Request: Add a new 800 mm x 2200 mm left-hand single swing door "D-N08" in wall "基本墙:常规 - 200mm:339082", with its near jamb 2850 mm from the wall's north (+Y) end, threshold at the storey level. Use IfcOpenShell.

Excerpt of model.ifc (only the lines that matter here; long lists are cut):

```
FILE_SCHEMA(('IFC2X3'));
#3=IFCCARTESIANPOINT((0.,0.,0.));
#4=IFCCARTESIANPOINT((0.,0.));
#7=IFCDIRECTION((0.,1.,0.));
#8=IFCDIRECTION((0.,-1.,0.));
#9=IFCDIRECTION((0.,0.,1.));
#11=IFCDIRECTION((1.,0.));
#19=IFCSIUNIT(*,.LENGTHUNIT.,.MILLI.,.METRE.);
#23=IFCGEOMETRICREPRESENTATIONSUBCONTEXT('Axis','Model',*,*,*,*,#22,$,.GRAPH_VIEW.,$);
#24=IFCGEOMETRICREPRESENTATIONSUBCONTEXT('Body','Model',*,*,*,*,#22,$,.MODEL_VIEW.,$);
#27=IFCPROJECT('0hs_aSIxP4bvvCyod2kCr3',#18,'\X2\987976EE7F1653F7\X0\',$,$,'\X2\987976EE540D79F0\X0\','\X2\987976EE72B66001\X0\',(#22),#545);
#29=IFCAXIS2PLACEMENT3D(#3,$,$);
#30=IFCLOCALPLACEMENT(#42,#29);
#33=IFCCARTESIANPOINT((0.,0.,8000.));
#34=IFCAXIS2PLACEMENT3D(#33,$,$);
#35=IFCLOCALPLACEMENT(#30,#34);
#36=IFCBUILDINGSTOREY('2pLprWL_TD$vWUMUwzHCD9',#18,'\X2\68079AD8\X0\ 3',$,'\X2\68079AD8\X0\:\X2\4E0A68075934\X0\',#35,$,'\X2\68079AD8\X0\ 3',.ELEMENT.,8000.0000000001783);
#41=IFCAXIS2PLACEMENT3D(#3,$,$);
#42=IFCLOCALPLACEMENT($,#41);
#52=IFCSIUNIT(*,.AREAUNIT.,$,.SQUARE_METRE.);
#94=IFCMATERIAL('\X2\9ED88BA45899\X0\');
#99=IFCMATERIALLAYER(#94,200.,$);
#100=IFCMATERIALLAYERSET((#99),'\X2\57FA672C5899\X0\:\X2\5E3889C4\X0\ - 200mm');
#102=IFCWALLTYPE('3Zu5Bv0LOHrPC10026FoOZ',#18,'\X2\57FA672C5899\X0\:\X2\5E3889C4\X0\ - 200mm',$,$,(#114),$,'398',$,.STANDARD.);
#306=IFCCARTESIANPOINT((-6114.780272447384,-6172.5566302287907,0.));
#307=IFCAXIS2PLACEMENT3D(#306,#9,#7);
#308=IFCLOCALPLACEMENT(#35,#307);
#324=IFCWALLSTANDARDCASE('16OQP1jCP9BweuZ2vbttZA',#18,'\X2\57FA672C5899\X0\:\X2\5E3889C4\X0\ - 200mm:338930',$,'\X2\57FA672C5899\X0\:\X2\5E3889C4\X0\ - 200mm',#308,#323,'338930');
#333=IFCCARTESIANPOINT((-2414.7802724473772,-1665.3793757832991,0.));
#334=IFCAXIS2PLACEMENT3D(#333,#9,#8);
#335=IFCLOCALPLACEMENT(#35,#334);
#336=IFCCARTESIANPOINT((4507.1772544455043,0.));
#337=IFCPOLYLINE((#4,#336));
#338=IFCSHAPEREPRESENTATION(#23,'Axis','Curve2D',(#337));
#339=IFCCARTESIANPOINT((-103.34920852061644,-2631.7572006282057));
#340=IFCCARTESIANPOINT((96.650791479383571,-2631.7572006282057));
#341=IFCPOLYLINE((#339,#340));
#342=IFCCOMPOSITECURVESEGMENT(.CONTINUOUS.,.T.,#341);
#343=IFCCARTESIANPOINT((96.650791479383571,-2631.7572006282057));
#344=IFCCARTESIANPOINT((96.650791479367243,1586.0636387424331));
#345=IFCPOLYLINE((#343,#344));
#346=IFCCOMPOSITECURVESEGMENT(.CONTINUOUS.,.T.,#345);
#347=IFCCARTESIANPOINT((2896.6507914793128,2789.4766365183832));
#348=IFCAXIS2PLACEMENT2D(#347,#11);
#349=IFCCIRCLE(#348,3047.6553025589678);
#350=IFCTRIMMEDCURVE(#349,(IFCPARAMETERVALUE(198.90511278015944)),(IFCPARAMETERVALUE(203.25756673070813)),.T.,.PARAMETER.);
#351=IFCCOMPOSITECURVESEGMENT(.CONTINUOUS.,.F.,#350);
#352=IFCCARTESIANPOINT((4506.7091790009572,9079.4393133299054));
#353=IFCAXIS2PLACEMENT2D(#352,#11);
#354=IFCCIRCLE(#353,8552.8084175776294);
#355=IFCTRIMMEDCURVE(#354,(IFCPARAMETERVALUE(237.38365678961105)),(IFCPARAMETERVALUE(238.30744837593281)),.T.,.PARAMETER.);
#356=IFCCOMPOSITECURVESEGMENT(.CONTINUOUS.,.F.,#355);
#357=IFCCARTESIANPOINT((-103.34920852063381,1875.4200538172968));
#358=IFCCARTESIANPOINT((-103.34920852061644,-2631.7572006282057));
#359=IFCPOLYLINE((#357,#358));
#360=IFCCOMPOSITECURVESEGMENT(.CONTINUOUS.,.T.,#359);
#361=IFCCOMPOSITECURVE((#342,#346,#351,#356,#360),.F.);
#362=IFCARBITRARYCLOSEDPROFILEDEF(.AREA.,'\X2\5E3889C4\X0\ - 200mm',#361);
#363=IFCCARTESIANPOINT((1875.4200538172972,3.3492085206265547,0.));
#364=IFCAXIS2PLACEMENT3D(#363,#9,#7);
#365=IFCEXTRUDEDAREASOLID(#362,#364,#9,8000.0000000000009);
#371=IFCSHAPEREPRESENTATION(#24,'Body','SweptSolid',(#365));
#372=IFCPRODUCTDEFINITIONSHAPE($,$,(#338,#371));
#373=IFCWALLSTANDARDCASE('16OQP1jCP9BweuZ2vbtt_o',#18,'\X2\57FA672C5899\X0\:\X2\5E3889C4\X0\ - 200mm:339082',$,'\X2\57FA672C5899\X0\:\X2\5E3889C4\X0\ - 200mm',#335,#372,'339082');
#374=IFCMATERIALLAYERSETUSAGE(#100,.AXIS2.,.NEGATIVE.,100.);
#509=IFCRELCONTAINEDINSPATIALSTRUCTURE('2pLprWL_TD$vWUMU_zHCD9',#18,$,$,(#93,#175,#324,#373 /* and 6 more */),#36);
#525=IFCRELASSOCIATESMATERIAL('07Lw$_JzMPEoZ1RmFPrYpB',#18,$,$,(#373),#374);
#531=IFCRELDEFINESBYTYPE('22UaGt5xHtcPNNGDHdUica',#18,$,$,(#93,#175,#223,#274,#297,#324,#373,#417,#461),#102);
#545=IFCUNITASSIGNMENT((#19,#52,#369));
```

```python
import numpy as np
import ifcopenshell
import ifcopenshell.api.feature
import ifcopenshell.api.geometry
import ifcopenshell.api.root
import ifcopenshell.api.spatial
import ifcopenshell.api.type
import ifcopenshell.geom
import ifcopenshell.util.element
import ifcopenshell.util.placement
import ifcopenshell.util.representation
import ifcopenshell.util.shape
import ifcopenshell.util.unit

model = ifcopenshell.open("model.ifc")
unit_scale = ifcopenshell.util.unit.calculate_unit_scale(model)
settings = ifcopenshell.geom.settings()


def volume(element):
    """Net volume in cubic metres, openings subtracted."""
    shape = ifcopenshell.geom.create_shape(settings, element)
    return ifcopenshell.util.shape.get_volume(shape.geometry)


wall = model.by_guid("16OQP1jCP9BweuZ2vbtt_o")
storey = ifcopenshell.util.element.get_container(wall, ifc_class="IfcBuildingStorey")
context = ifcopenshell.util.representation.get_context(model, "Model", "Body", "MODEL_VIEW")
before = volume(wall)

width, height, from_end, sill = 0.8, 2.2, 2.85, 0.0  # metres

# The wall runs along its own X axis, and the end named is its -X end.
wall_shape = ifcopenshell.geom.create_shape(settings, wall)
x, y, z = ifcopenshell.util.shape.get_vertices(wall_shape.geometry).T
start = x.min() + from_end
face, thickness = float(y.min()), float(y.max() - y.min())
wall_matrix = ifcopenshell.util.placement.get_local_placement(wall.ObjectPlacement)
level = ifcopenshell.util.placement.get_local_placement(storey.ObjectPlacement)[2, 3]


def in_wall(x, y):
    """Placement at x, y metres in the wall's axes, at sill height."""
    matrix = wall_matrix.copy()
    matrix[:, 3] = wall_matrix @ np.array([x / unit_scale, y / unit_scale, 0.0, 1.0])
    matrix[2, 3] = level + sill / unit_scale
    return matrix


# Opening: a box that overshoots both wall faces by 50 mm.
opening = ifcopenshell.api.root.create_entity(model, ifc_class="IfcOpeningElement")
box = ifcopenshell.api.geometry.add_wall_representation(
    model, context=context, length=width, height=height, thickness=thickness + 0.1
)
ifcopenshell.api.geometry.assign_representation(model, product=opening, representation=box)
ifcopenshell.api.geometry.edit_object_placement(model, product=opening, matrix=in_wall(start, face - 0.05), is_si=False)
ifcopenshell.api.feature.add_feature(model, feature=opening, element=wall)

door = ifcopenshell.api.root.create_entity(model, ifc_class="IfcDoor", name="D-N08")
door.OverallWidth, door.OverallHeight = width / unit_scale, height / unit_scale
body = ifcopenshell.api.geometry.add_door_representation(
    model,
    context=context,
    overall_width=door.OverallWidth,
    overall_height=door.OverallHeight,
    operation_type="SINGLE_SWING_LEFT",
    lining_properties={"LiningDepth": thickness / unit_scale, "ThresholdDepth": thickness / unit_scale},
)
ifcopenshell.api.geometry.assign_representation(model, product=door, representation=body)
ifcopenshell.api.spatial.assign_container(model, products=[door], relating_structure=storey)
fills = ifcopenshell.api.feature.add_filling(model, opening=opening, element=door)
fills.OwnerHistory = door.OwnerHistory  # required in IFC2X3

# IFC2X3 keeps the operation on the door style.
style = ifcopenshell.api.root.create_entity(model, ifc_class="IfcDoorStyle", name="D-N08")
style.OperationType, style.ConstructionType = "SINGLE_SWING_LEFT", "NOTDEFINED"
style.ParameterTakesPrecedence = style.Sizeable = False
ifcopenshell.api.type.assign_type(model, related_objects=[door], relating_type=style)

# The lining spans the wall, so the door starts at the wall face.
ifcopenshell.api.geometry.edit_object_placement(model, product=door, matrix=in_wall(start, face), is_si=False)

after = volume(wall)

print(f"wall volume {before:.3f} -> {after:.3f} m3")

model.write("model_v2.ifc")
```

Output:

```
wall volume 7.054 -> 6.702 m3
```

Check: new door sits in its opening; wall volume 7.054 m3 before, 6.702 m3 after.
